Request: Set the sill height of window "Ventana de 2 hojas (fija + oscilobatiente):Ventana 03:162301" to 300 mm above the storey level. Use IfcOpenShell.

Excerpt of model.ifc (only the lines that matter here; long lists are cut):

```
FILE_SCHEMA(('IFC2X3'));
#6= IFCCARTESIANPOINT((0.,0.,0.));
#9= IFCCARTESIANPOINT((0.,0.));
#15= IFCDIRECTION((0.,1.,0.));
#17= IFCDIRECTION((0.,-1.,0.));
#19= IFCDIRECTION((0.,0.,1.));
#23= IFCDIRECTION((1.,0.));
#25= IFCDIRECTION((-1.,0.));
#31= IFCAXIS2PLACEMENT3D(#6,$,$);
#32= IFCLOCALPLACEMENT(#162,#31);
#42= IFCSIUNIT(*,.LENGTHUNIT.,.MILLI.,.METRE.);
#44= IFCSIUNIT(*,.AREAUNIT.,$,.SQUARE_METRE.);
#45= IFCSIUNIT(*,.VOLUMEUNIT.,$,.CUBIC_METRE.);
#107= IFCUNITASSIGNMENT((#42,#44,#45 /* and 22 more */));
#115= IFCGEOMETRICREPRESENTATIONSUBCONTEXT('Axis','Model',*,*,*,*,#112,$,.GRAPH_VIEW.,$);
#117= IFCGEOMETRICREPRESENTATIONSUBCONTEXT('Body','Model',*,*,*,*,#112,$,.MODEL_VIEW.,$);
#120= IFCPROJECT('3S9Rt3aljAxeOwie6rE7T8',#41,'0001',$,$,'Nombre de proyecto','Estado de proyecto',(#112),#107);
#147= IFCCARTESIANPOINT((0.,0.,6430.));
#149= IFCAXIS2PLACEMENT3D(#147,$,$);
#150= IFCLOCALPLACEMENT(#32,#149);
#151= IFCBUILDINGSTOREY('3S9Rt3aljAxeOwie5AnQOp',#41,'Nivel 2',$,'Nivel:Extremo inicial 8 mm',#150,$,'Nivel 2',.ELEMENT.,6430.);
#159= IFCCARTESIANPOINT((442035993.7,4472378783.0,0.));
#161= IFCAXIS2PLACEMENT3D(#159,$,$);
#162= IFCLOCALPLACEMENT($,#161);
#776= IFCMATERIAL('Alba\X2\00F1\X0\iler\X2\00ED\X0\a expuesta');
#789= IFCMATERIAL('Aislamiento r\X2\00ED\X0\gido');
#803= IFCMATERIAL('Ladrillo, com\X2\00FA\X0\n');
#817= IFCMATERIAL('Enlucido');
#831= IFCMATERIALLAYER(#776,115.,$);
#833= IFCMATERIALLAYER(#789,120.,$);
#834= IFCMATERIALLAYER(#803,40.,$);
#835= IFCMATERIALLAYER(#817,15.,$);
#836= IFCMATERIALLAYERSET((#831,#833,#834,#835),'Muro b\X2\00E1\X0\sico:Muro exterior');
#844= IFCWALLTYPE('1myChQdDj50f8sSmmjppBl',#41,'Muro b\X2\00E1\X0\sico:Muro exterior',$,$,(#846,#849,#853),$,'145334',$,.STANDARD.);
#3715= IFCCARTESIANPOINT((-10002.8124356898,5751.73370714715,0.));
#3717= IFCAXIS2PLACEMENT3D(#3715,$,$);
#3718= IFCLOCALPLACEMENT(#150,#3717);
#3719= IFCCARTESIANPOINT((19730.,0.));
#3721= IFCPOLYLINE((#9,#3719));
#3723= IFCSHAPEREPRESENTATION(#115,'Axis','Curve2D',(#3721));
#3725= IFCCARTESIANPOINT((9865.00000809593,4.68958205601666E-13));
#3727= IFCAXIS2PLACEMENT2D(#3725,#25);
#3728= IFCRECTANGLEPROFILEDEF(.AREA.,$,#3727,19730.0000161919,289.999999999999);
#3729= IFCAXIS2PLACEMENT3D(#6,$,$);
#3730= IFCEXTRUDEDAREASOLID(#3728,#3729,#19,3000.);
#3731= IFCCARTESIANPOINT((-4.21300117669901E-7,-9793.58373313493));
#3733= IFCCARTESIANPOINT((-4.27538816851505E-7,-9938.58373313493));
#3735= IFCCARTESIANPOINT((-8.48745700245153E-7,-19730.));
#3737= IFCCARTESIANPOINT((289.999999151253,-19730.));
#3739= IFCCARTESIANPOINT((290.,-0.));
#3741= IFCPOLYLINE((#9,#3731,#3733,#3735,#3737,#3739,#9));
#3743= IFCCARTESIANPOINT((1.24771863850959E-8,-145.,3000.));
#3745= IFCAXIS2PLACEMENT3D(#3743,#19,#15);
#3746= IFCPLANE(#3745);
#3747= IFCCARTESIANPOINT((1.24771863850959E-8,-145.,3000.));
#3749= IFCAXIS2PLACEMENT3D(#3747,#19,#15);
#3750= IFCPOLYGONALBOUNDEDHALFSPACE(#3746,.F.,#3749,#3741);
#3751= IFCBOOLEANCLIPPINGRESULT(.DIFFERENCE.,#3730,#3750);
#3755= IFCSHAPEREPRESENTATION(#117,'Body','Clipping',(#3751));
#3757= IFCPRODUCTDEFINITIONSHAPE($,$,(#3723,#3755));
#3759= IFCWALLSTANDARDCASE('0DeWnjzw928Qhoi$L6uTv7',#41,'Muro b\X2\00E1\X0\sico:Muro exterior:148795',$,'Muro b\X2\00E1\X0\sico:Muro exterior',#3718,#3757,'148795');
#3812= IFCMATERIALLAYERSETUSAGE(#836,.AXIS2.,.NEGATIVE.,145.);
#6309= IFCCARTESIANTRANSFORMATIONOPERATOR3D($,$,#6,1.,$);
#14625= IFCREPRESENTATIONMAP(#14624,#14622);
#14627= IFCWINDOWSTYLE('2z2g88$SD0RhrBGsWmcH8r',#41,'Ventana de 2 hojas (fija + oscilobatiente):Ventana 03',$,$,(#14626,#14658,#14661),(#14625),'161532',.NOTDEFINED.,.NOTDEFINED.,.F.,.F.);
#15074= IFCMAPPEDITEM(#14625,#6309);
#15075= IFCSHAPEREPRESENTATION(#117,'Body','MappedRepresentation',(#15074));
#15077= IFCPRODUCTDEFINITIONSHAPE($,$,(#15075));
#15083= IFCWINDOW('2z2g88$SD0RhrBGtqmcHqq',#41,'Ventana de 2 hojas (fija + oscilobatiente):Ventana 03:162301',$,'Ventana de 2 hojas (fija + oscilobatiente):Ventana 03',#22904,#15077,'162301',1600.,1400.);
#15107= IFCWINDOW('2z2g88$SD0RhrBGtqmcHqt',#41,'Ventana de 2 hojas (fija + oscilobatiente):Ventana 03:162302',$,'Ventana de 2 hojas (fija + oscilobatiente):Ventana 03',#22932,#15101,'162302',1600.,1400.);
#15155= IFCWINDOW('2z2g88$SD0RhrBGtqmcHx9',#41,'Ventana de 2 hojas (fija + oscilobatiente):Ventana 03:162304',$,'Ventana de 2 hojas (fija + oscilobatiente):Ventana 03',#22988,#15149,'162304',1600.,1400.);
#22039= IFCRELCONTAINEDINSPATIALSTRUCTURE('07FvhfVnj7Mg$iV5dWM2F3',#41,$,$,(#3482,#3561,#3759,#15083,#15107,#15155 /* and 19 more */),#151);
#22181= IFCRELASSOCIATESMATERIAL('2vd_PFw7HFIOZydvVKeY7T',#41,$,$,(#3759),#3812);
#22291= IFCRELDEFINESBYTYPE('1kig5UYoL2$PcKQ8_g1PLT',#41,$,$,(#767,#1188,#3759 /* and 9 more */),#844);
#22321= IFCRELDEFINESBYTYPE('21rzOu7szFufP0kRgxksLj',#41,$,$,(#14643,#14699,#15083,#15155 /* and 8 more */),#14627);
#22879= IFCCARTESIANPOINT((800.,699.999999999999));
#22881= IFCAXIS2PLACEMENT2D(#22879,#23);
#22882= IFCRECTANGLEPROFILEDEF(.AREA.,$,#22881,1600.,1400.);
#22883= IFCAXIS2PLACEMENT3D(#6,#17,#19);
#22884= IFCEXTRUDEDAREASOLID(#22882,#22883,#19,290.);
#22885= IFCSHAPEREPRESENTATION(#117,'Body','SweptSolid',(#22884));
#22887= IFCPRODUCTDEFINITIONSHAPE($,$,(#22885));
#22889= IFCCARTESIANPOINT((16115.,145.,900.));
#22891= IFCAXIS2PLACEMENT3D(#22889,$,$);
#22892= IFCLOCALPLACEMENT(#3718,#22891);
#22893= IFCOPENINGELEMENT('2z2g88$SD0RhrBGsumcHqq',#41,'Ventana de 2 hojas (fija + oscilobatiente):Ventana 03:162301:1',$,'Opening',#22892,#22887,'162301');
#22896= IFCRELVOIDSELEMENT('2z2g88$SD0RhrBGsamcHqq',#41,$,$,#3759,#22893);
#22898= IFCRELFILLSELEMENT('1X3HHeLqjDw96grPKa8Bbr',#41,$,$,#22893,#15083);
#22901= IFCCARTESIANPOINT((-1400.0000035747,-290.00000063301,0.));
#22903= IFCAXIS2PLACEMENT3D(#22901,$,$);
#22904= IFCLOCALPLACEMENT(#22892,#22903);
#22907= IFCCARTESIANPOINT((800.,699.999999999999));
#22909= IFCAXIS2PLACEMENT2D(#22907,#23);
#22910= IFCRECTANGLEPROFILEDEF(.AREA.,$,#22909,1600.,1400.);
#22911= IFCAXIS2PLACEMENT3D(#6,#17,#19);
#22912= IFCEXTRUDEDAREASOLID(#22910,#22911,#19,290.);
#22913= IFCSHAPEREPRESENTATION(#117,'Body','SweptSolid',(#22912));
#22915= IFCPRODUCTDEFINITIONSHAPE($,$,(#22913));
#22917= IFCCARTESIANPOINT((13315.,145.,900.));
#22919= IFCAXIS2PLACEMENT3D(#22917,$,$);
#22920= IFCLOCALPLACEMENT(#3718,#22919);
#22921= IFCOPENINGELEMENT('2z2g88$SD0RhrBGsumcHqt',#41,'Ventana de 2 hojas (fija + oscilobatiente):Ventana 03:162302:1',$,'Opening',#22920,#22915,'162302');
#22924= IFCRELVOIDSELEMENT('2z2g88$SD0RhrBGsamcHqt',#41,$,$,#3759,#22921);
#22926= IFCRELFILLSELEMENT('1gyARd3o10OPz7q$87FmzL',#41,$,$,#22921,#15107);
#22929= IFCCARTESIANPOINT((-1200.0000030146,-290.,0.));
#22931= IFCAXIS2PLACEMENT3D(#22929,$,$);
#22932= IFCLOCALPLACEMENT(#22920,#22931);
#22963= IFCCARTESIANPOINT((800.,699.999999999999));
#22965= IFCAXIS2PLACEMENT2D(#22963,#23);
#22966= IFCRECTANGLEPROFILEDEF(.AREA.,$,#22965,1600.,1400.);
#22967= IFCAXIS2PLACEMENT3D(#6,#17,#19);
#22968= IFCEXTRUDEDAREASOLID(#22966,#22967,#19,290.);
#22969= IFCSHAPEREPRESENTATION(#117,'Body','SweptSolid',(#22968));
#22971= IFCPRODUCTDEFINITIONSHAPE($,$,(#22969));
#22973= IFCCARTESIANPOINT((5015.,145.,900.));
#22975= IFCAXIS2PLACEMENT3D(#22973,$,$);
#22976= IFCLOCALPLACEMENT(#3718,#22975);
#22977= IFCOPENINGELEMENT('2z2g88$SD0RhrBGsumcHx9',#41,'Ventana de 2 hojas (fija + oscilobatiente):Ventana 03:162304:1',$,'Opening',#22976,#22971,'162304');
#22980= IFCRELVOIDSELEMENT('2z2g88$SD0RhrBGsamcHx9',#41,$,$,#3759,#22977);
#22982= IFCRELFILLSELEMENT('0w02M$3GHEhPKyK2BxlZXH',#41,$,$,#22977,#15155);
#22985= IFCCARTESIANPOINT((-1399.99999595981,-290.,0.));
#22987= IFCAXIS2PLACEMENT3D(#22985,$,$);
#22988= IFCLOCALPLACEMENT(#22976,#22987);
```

```python
import numpy as np
import ifcopenshell
import ifcopenshell.api.geometry
import ifcopenshell.geom
import ifcopenshell.util.element
import ifcopenshell.util.placement
import ifcopenshell.util.shape
import ifcopenshell.util.unit

model = ifcopenshell.open("model.ifc")
unit_scale = ifcopenshell.util.unit.calculate_unit_scale(model)

window = model.by_guid("2z2g88$SD0RhrBGtqmcHqq")
opening = window.FillsVoids[0].RelatingOpeningElement
storey = ifcopenshell.util.element.get_container(window, ifc_class="IfcBuildingStorey")
level = ifcopenshell.util.placement.get_local_placement(storey.ObjectPlacement)[2, 3]

# The opening's origin need not be at the sill, so measure its lowest point.
shape = ifcopenshell.geom.create_shape(ifcopenshell.geom.settings(), opening)
bottom = ifcopenshell.util.shape.get_shape_bottom_elevation(shape, shape.geometry) / unit_scale
dz = level + 0.3 / unit_scale - bottom

shift = np.array([0.0, 0.0, dz])
# The window is placed relative to its opening, so it follows when the opening moves.
matrix = ifcopenshell.util.placement.get_local_placement(opening.ObjectPlacement)
matrix[:3, 3] += shift
ifcopenshell.api.geometry.edit_object_placement(
    model, product=opening, matrix=matrix, is_si=False, should_transform_children=True
)

print(f"moved by {dz * unit_scale:+.3f} m")

model.write("model_v2.ifc")
```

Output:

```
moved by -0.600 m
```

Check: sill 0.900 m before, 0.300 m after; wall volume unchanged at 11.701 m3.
